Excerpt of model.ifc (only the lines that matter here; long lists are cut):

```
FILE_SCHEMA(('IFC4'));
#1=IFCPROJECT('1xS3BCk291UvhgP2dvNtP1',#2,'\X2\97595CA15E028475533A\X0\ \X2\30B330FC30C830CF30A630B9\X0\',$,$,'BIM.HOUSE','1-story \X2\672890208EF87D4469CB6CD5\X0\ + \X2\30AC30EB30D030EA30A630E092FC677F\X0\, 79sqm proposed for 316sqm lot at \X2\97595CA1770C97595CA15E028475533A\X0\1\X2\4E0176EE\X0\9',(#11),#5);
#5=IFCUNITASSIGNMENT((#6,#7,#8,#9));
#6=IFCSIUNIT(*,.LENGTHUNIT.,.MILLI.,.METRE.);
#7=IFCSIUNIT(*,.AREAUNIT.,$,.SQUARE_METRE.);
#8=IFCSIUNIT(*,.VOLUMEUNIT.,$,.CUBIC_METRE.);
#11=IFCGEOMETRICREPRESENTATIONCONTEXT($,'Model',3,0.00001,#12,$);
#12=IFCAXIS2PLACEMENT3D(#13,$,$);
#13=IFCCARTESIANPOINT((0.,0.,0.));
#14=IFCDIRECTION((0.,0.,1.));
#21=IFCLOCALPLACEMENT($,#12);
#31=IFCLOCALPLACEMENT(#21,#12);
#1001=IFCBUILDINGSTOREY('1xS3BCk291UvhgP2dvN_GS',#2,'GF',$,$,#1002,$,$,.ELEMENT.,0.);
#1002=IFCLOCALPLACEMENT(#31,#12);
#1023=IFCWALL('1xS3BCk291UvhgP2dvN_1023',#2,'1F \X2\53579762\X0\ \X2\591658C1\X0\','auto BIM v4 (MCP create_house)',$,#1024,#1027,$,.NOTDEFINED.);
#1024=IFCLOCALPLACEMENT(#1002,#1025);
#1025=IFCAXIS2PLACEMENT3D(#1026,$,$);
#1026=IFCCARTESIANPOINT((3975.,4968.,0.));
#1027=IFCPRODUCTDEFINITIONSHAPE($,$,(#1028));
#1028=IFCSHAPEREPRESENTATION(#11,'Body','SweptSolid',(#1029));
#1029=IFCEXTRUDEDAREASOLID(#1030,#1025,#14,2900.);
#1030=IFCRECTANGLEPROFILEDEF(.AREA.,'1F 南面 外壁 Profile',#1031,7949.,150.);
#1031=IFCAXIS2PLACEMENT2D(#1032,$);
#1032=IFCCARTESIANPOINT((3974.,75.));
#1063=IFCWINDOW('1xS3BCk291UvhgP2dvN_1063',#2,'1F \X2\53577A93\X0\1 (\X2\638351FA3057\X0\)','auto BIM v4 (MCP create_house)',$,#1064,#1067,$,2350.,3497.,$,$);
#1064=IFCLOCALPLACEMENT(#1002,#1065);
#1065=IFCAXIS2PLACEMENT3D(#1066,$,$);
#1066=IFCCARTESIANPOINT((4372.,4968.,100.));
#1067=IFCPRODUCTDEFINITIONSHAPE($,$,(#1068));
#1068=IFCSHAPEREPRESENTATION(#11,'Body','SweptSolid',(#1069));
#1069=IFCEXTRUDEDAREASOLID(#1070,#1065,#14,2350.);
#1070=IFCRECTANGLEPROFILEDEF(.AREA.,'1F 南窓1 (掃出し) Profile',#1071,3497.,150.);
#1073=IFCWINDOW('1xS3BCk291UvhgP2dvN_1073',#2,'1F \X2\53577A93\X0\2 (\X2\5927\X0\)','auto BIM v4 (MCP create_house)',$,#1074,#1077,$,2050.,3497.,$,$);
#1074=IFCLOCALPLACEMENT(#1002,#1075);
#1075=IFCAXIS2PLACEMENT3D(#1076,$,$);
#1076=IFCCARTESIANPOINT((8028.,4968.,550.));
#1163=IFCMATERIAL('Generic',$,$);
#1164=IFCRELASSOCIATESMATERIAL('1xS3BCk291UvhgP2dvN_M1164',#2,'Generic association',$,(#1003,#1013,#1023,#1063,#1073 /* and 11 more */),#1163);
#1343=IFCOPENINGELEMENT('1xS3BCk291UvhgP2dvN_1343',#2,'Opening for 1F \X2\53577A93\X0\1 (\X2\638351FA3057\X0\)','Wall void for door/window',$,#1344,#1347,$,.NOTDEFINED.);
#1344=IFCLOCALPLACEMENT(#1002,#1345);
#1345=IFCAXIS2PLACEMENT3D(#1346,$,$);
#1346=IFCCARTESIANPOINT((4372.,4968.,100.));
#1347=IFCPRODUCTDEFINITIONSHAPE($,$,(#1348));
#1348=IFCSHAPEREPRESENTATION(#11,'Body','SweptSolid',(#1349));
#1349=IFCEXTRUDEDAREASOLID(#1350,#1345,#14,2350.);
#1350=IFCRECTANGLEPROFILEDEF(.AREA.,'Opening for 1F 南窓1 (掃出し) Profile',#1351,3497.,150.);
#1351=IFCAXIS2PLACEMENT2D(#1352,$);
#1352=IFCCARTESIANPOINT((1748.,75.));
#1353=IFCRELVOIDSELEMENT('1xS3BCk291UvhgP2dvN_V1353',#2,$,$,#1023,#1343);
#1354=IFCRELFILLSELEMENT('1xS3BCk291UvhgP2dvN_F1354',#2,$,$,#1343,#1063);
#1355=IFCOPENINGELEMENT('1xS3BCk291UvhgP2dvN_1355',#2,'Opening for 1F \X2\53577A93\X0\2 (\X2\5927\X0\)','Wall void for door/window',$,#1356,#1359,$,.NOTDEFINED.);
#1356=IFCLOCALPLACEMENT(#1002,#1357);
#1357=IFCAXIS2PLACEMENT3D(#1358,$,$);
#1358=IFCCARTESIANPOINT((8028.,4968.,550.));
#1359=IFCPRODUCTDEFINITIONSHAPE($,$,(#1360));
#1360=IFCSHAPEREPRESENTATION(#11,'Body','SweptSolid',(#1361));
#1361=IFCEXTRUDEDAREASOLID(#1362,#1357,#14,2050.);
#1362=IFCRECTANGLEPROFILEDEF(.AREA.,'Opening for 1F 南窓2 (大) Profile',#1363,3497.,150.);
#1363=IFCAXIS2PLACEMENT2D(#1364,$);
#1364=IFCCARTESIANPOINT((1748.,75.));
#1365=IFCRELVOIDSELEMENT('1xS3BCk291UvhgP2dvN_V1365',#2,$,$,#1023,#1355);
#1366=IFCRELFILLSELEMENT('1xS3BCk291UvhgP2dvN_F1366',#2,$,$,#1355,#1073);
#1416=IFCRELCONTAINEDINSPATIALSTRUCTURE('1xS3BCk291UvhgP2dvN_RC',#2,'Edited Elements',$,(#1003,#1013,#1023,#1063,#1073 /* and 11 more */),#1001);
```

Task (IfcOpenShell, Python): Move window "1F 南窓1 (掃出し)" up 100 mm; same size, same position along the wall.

```python
import numpy as np
import ifcopenshell
import ifcopenshell.api.geometry
import ifcopenshell.util.placement
import ifcopenshell.util.unit

model = ifcopenshell.open("model.ifc")
unit_scale = ifcopenshell.util.unit.calculate_unit_scale(model)

window = model.by_guid("1xS3BCk291UvhgP2dvN_1063")
opening = window.FillsVoids[0].RelatingOpeningElement
dz = 0.1 / unit_scale

shift = np.array([0.0, 0.0, dz])
# The window is not placed relative to its opening, so move both.
for product in (opening, window):
    matrix = ifcopenshell.util.placement.get_local_placement(product.ObjectPlacement)
    matrix[:3, 3] += shift
    ifcopenshell.api.geometry.edit_object_placement(model, product=product, matrix=matrix, is_si=False)

print(f"moved by {dz * unit_scale:+.3f} m")

model.write("model_updated.ifc")
```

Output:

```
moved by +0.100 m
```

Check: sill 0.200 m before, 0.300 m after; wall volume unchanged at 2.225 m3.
